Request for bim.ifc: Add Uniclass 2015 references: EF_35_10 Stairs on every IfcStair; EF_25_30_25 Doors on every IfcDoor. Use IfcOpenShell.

First a look at what the model holds.

```python
import ifcopenshell

model = ifcopenshell.open("bim.ifc")
print(model.schema)
print("classifications:", [c.Name for c in model.by_type("IfcClassification")])
for ifc_class in ("IfcDoor", "IfcRoof", "IfcStair", "IfcWall", "IfcWindow"):
    print(ifc_class, len(model.by_type(ifc_class)))
```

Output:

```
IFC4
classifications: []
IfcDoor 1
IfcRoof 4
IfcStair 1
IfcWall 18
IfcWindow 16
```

```python
import ifcopenshell
import ifcopenshell.api.classification

model = ifcopenshell.open("bim.ifc")

system = ifcopenshell.api.classification.add_classification(model, classification="Uniclass 2015")

codes = {
    "IfcStair": ("EF_35_10", "Stairs"),
    "IfcDoor": ("EF_25_30_25", "Doors"),
}
for ifc_class, (code, name) in codes.items():
    products = model.by_type(ifc_class)
    ifcopenshell.api.classification.add_reference(
        model, products=products, classification=system, identification=code, name=name
    )
    print(code, len(products))

model.write("bim_updated.ifc")
```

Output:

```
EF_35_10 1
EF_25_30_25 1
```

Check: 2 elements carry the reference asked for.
